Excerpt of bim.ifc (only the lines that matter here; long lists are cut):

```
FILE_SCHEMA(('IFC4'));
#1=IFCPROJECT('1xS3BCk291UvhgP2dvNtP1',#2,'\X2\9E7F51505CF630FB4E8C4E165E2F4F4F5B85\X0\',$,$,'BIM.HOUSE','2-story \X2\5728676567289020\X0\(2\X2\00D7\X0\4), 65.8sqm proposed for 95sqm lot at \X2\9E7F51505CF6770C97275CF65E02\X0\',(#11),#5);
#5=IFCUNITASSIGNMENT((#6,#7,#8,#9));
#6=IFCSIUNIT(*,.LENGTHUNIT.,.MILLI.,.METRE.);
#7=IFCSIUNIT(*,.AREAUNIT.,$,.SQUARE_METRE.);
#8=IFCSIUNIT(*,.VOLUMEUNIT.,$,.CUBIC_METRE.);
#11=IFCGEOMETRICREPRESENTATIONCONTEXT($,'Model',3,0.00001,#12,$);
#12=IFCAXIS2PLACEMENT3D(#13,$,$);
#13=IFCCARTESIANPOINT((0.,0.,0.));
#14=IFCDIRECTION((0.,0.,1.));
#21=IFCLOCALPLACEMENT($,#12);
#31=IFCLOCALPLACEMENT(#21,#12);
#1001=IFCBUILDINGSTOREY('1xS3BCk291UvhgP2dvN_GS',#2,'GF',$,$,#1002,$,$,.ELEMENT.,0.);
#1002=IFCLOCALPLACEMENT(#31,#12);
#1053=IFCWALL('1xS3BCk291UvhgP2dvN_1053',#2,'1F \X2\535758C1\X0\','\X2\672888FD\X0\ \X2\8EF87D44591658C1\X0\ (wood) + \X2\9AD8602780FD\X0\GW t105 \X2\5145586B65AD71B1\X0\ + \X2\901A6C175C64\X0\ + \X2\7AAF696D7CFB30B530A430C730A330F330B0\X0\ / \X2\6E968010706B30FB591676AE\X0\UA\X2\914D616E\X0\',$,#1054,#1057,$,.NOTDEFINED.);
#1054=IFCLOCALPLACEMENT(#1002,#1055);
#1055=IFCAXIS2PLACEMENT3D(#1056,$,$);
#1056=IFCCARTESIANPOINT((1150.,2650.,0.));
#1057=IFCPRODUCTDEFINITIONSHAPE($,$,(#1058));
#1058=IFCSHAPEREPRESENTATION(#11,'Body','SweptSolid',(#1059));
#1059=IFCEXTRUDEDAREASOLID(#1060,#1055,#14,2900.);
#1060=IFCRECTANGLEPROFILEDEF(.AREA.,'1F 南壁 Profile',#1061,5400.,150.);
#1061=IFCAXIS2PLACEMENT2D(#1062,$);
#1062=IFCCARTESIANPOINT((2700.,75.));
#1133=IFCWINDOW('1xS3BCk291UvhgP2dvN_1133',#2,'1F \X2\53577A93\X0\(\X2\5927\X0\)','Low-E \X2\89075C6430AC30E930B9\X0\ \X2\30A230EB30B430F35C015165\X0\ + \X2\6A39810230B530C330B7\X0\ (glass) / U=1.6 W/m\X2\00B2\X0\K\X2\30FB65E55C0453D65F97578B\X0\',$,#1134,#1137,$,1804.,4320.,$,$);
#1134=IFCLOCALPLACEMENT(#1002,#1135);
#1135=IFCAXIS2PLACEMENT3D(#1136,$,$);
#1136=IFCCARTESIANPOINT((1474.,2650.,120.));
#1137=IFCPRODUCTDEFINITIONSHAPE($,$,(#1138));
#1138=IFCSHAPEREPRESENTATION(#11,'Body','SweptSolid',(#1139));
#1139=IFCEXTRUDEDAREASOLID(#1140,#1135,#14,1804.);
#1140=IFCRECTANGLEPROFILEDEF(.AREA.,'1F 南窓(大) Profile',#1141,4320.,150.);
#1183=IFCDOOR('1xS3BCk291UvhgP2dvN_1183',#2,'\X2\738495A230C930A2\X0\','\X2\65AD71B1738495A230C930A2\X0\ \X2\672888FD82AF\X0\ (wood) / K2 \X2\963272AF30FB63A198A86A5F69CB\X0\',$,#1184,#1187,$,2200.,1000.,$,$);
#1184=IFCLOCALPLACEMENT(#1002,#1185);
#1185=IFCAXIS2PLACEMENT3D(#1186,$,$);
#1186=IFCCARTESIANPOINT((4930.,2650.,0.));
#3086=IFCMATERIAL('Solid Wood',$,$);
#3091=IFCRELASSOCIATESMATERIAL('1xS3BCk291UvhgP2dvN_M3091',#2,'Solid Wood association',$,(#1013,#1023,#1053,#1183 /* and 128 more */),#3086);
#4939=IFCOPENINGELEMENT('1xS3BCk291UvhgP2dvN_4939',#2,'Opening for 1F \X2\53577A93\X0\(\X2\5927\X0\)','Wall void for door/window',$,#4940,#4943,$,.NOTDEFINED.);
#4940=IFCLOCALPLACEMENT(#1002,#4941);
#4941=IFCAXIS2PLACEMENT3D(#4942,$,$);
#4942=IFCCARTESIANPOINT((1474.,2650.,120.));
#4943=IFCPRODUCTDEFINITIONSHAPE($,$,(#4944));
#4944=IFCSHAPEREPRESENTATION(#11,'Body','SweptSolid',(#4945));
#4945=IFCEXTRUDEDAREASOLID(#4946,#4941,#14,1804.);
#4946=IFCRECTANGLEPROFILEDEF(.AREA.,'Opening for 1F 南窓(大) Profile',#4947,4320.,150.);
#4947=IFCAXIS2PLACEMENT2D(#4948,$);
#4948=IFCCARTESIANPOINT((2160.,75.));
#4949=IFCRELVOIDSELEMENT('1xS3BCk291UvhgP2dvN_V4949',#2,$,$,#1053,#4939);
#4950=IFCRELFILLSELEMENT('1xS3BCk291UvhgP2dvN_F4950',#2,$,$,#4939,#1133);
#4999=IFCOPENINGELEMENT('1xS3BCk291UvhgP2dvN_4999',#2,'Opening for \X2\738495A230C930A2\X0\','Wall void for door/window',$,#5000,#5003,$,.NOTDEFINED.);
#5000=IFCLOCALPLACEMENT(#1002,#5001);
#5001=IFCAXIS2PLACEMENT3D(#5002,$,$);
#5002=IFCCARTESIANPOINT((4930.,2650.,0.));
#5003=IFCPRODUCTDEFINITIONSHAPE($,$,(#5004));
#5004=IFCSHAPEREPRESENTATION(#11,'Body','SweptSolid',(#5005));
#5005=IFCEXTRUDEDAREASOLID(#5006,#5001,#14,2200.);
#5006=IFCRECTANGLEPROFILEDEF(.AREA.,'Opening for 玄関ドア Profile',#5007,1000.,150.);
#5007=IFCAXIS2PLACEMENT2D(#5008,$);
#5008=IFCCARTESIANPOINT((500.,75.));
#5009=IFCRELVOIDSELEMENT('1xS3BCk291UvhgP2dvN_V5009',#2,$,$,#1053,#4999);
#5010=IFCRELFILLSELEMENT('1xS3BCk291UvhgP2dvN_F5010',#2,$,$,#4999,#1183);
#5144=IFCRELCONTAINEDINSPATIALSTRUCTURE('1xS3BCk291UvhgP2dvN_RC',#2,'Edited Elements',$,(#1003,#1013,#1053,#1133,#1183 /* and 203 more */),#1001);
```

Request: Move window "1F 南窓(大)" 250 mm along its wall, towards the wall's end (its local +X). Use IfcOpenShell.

```python
import ifcopenshell
import ifcopenshell.api.geometry
import ifcopenshell.util.placement

model = ifcopenshell.open("bim.ifc")

window = model.by_guid("1xS3BCk291UvhgP2dvN_1133")
opening = window.FillsVoids[0].RelatingOpeningElement
wall = opening.VoidsElements[0].RelatingBuildingElement

wall_matrix = ifcopenshell.util.placement.get_local_placement(wall.ObjectPlacement)
shift = wall_matrix[:3, 0] * 250.0
before = ifcopenshell.util.placement.get_local_placement(window.ObjectPlacement)[:3, 3].copy()

# The window is not placed relative to its opening, so move both.
for product in (opening, window):
    matrix = ifcopenshell.util.placement.get_local_placement(product.ObjectPlacement)
    matrix[:3, 3] += shift
    ifcopenshell.api.geometry.edit_object_placement(model, product=product, matrix=matrix, is_si=False)

after = ifcopenshell.util.placement.get_local_placement(window.ObjectPlacement)[:3, 3]
print("window moved by", (after - before).round(3) + 0.0)

model.write("bim_edited.ifc")
```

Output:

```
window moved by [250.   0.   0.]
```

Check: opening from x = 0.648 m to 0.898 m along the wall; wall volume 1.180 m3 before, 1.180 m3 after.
